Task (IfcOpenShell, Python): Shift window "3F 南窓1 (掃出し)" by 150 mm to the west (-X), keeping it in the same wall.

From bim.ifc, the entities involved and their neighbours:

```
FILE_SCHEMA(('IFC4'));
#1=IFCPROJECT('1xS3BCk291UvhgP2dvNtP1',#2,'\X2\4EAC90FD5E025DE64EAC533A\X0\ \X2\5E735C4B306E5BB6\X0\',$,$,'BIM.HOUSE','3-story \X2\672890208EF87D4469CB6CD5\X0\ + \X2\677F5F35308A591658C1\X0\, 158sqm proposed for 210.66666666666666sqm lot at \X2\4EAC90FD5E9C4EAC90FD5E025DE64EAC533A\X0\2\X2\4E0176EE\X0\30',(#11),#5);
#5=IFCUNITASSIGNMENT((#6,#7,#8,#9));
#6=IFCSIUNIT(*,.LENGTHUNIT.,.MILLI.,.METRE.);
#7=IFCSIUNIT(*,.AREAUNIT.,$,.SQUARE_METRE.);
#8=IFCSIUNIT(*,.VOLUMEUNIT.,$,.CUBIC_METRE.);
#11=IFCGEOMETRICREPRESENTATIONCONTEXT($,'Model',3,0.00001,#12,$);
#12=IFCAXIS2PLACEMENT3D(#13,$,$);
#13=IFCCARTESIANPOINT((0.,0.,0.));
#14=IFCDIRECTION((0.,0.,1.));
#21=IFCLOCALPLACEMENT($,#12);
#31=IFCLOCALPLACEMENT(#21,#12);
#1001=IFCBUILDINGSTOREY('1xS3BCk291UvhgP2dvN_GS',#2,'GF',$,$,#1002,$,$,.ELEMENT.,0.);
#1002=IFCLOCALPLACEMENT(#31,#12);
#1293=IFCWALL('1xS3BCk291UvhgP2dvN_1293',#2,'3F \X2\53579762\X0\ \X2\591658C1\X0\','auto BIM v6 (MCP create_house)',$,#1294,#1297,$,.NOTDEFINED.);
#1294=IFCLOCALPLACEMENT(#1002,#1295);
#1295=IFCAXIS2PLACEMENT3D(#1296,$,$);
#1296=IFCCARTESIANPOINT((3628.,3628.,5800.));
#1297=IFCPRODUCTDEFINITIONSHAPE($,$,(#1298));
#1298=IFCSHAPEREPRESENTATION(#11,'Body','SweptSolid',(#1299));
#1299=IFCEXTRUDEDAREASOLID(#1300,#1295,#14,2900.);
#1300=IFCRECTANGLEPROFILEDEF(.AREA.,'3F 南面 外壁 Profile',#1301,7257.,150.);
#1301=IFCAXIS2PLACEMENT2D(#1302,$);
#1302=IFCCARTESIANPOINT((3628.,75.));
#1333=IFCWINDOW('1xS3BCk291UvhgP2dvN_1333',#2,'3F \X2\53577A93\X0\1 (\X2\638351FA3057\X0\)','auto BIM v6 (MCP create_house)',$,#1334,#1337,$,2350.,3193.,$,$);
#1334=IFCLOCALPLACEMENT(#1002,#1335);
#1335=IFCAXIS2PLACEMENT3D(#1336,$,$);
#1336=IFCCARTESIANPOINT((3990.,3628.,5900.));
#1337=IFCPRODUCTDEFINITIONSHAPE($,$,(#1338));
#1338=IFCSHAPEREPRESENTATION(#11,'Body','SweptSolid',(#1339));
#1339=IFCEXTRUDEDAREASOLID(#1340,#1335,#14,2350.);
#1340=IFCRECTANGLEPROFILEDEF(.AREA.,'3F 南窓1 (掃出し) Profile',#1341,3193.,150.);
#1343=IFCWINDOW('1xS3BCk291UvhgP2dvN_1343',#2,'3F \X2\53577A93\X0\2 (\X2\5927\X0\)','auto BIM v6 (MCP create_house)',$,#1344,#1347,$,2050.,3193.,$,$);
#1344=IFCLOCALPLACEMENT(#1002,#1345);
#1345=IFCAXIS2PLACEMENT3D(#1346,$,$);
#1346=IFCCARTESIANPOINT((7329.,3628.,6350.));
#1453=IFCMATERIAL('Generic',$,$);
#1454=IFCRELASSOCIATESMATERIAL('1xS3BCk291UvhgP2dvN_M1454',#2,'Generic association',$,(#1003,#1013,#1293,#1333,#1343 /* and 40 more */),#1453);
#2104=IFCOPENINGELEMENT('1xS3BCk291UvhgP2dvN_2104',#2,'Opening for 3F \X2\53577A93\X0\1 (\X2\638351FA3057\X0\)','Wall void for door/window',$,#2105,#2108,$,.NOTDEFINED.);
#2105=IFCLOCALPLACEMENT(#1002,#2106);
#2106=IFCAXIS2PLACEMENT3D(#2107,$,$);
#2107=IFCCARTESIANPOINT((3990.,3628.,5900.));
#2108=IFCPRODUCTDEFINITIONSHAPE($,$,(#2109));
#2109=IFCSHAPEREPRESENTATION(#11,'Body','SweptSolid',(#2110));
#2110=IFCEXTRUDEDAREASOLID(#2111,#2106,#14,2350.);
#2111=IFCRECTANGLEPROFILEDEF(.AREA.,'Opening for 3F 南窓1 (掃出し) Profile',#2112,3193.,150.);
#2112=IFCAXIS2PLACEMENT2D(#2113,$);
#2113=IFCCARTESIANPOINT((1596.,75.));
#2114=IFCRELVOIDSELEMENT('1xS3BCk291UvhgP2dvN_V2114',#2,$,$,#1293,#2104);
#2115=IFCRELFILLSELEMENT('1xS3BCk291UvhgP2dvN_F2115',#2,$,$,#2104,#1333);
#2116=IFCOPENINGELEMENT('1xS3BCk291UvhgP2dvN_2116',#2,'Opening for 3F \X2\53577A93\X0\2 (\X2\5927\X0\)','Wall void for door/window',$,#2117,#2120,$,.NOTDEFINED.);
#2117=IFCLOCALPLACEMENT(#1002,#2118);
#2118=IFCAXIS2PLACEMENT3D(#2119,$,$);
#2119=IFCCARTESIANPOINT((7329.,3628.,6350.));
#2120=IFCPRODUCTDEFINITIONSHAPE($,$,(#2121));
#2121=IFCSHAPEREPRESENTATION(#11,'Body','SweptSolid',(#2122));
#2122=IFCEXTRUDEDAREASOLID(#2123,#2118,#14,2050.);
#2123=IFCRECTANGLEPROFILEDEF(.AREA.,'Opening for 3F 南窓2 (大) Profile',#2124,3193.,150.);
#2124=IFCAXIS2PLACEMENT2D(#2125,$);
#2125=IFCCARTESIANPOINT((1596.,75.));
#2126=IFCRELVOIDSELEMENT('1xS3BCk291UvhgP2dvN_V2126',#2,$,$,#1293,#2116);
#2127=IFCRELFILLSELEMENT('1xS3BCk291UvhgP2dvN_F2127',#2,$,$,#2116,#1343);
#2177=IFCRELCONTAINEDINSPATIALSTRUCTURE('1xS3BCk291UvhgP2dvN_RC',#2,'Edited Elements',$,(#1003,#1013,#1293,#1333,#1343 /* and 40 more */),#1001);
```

```python
import ifcopenshell
import ifcopenshell.api.geometry
import ifcopenshell.util.placement
import ifcopenshell.util.unit

model = ifcopenshell.open("bim.ifc")
unit_scale = ifcopenshell.util.unit.calculate_unit_scale(model)

window = model.by_guid("1xS3BCk291UvhgP2dvN_1333")
opening = window.FillsVoids[0].RelatingOpeningElement
wall = opening.VoidsElements[0].RelatingBuildingElement

wall_matrix = ifcopenshell.util.placement.get_local_placement(wall.ObjectPlacement)
shift = wall_matrix[:3, 0] * -0.15 / unit_scale
before = ifcopenshell.util.placement.get_local_placement(window.ObjectPlacement)[:3, 3].copy()

# The window is not placed relative to its opening, so move both.
for product in (opening, window):
    matrix = ifcopenshell.util.placement.get_local_placement(product.ObjectPlacement)
    matrix[:3, 3] += shift
    ifcopenshell.api.geometry.edit_object_placement(model, product=product, matrix=matrix, is_si=False)

after = ifcopenshell.util.placement.get_local_placement(window.ObjectPlacement)[:3, 3]
print("window moved by", (after - before).round(3) + 0.0)

model.write("bim_edited.ifc")
```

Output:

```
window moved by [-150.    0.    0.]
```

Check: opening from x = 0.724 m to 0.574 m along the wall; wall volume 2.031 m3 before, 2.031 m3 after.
